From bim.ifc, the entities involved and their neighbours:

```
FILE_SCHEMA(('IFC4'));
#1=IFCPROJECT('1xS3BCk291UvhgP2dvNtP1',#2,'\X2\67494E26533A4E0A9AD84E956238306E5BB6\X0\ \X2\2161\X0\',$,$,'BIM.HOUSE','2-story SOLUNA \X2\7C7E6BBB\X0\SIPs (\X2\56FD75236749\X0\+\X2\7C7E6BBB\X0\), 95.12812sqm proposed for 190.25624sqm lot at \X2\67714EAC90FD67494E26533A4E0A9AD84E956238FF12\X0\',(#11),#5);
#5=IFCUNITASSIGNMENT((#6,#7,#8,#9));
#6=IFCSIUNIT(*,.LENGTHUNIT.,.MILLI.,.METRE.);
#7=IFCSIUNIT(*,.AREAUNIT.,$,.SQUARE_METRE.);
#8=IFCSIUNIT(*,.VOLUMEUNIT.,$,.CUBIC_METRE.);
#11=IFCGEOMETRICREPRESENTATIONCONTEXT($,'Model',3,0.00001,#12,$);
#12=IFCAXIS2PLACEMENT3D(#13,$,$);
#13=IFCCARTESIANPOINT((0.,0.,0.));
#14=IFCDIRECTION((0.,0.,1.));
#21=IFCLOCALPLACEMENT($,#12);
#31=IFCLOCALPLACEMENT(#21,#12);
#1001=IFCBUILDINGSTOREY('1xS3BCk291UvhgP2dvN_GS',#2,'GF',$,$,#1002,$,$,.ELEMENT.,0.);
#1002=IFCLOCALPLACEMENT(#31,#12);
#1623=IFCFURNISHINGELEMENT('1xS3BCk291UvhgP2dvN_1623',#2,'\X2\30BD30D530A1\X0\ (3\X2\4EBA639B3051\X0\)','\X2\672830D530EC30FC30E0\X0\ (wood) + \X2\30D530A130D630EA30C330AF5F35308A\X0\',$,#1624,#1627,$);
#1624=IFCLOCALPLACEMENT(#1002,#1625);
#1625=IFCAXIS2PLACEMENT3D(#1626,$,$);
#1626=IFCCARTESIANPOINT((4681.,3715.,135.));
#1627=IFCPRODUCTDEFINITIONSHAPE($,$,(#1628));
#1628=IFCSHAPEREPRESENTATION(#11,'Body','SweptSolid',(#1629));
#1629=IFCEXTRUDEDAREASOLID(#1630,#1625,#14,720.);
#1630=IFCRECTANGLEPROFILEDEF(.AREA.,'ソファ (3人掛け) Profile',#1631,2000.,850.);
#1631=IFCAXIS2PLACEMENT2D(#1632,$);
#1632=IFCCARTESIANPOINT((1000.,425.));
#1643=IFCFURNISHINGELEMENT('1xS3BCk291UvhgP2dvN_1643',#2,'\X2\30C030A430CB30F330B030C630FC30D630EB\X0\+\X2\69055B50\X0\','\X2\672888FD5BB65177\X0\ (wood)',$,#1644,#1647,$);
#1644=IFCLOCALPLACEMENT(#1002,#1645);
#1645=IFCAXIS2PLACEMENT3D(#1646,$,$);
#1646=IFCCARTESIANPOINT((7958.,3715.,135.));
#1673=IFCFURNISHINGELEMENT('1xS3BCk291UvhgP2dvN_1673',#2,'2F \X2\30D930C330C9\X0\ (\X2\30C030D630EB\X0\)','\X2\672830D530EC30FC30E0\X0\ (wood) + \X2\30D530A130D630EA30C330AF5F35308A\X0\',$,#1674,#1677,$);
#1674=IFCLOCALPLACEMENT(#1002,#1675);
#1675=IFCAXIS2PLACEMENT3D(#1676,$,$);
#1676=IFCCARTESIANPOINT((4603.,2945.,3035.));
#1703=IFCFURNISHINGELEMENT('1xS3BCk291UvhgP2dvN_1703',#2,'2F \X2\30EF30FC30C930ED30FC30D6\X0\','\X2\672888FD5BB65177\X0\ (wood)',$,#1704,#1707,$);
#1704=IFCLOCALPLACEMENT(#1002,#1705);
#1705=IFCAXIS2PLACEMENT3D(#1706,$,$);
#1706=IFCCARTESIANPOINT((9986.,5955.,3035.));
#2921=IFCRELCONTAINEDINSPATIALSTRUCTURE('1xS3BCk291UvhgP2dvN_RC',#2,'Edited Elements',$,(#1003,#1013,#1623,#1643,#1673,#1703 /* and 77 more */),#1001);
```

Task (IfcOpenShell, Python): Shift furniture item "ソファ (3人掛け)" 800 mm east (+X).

```python
import ifcopenshell
import ifcopenshell.api.geometry
import ifcopenshell.util.placement
import ifcopenshell.util.unit

model = ifcopenshell.open("bim.ifc")
unit_scale = ifcopenshell.util.unit.calculate_unit_scale(model)

item = model.by_id(1623)
matrix = ifcopenshell.util.placement.get_local_placement(item.ObjectPlacement)
matrix[0, 3] += 0.8 / unit_scale
ifcopenshell.api.geometry.edit_object_placement(model, product=item, matrix=matrix, is_si=False)

print(ifcopenshell.util.placement.get_local_placement(item.ObjectPlacement).round(3) + 0.0)

model.write("bim_rev.ifc")
```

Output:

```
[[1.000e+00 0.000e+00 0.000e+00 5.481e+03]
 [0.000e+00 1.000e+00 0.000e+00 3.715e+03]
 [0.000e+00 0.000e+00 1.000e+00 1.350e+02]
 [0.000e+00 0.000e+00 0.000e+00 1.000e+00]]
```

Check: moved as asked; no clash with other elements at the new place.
